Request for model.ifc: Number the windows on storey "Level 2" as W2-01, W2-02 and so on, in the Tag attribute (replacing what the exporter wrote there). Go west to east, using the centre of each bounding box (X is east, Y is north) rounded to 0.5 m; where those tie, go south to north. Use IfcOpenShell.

First a look at what the model holds.

```python
import ifcopenshell
import ifcopenshell.util.element
import ifcopenshell.util.placement

model = ifcopenshell.open("model.ifc")
print(model.schema)
storey = next(s for s in model.by_type("IfcBuildingStorey") if s.Name == "Level 2")
windows = [e for e in ifcopenshell.util.element.get_decomposition(storey) if e.is_a("IfcWindow")]
for e in sorted(windows, key=lambda e: e.id()):
    origin = ifcopenshell.util.placement.get_local_placement(e.ObjectPlacement)[:3, 3]
    print(e.id(), e.Tag, e.Name, origin.round(2) + 0.0, sep=" | ")
```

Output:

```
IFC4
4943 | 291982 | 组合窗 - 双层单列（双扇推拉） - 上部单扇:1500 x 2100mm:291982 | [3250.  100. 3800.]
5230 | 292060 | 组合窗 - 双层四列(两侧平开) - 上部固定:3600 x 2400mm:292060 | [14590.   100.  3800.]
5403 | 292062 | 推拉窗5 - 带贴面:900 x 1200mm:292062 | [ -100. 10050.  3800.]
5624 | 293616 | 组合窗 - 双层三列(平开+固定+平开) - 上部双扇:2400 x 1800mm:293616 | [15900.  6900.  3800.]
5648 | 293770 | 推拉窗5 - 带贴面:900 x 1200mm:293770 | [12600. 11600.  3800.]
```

```python
import ifcopenshell
import ifcopenshell.geom
import ifcopenshell.util.element
import ifcopenshell.util.shape

model = ifcopenshell.open("model.ifc")
settings = ifcopenshell.geom.settings()
settings.set("use-world-coords", True)


def centre(element):
    shape = ifcopenshell.geom.create_shape(settings, element)
    return ifcopenshell.util.shape.get_bbox_centroid(shape.geometry)


storey = next(s for s in model.by_type("IfcBuildingStorey") if s.Name == "Level 2")
windows = [e for e in ifcopenshell.util.element.get_decomposition(storey) if e.is_a("IfcWindow")]

# Insertion points can sit at a corner or the storey origin, so sort by the geometry (in metres).
centres = {e: centre(e) for e in windows}
windows.sort(key=lambda e: (round(centres[e][0] / 0.5), centres[e][1]))

for i, e in enumerate(windows, start=1):
    number = f"W2-{i:02d}"
    e.Tag = number
    print(e.id(), number)

model.write("model_rev.ifc")
```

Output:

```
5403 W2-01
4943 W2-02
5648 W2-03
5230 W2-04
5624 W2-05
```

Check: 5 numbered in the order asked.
